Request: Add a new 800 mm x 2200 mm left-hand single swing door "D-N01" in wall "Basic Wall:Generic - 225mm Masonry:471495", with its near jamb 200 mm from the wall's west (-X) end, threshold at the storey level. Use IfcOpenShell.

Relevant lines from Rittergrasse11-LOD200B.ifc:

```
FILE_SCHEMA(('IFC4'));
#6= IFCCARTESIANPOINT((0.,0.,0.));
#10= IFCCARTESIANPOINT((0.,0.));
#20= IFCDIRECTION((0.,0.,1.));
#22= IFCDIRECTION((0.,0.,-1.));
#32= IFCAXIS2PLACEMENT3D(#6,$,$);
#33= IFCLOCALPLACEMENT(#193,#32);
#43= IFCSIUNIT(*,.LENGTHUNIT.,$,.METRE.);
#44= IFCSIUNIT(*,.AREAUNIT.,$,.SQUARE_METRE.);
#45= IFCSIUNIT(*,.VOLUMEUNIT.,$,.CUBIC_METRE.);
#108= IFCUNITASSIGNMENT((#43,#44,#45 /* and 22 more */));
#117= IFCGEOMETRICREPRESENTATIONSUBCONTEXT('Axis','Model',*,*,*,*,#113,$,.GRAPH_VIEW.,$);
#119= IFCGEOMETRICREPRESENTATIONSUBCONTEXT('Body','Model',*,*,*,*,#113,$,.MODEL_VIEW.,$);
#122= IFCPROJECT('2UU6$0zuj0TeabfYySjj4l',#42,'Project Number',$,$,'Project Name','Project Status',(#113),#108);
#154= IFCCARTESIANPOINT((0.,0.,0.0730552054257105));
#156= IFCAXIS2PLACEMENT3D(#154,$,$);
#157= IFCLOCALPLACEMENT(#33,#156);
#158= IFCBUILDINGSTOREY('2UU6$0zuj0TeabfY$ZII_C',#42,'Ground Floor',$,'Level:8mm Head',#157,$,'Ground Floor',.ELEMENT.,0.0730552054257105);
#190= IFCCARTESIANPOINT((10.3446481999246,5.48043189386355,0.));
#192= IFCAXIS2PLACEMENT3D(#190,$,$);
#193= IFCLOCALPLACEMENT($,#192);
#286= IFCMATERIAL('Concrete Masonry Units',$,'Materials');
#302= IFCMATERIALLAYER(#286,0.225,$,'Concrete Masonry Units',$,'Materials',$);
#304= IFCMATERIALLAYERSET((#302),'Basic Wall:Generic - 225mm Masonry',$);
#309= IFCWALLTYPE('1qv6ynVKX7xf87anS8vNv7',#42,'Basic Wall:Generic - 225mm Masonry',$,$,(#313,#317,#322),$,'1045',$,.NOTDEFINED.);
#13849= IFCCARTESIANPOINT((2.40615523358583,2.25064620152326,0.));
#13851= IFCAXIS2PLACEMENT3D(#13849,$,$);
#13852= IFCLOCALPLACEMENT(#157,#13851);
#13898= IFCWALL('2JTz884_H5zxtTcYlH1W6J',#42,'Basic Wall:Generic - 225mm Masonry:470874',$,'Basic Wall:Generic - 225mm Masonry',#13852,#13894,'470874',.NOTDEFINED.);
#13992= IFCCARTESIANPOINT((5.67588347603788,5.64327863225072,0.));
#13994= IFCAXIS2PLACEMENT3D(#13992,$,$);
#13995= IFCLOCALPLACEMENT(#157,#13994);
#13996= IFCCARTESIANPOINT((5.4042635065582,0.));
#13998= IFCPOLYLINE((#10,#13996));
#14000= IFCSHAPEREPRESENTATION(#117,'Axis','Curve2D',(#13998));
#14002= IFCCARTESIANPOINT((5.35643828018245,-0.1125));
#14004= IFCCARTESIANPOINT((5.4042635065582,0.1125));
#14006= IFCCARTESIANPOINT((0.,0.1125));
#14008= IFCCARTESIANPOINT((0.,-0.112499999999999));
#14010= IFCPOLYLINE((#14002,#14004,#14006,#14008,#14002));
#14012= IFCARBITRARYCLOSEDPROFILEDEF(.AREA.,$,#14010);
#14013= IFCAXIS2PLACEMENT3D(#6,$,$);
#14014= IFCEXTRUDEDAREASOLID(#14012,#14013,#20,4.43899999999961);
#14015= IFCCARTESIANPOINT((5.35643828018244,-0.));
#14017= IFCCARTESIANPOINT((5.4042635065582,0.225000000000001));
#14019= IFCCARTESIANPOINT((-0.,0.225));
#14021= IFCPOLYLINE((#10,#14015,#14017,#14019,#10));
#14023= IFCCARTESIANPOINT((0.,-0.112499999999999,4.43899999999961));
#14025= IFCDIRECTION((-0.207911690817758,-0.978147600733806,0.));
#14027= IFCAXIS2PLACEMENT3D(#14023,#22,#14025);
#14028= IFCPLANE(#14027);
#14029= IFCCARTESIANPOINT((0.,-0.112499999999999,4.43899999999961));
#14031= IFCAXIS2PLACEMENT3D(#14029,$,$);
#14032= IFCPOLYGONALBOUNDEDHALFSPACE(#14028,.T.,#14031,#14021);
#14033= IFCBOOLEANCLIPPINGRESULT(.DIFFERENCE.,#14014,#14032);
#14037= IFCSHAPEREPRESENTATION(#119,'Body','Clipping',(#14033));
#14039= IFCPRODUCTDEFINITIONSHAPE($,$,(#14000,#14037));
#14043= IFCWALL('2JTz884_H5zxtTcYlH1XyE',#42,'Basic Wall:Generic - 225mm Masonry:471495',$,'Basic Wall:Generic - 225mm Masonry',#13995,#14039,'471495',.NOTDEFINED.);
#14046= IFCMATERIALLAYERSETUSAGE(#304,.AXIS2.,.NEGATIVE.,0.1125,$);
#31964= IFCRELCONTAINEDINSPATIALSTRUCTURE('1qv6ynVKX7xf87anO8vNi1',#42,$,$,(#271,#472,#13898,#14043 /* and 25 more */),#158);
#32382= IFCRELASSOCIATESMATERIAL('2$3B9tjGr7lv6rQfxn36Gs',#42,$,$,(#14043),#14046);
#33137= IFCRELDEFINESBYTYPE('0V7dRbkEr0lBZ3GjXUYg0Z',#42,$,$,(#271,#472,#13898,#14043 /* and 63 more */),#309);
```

```python
import numpy as np
import ifcopenshell
import ifcopenshell.api.feature
import ifcopenshell.api.geometry
import ifcopenshell.api.root
import ifcopenshell.api.spatial
import ifcopenshell.geom
import ifcopenshell.util.element
import ifcopenshell.util.placement
import ifcopenshell.util.representation
import ifcopenshell.util.shape
import ifcopenshell.util.unit

model = ifcopenshell.open("Rittergrasse11-LOD200B.ifc")
unit_scale = ifcopenshell.util.unit.calculate_unit_scale(model)
settings = ifcopenshell.geom.settings()


def volume(element):
    """Net volume in cubic metres, openings subtracted."""
    shape = ifcopenshell.geom.create_shape(settings, element)
    return ifcopenshell.util.shape.get_volume(shape.geometry)


wall = model.by_guid("2JTz884_H5zxtTcYlH1XyE")
storey = ifcopenshell.util.element.get_container(wall, ifc_class="IfcBuildingStorey")
context = ifcopenshell.util.representation.get_context(model, "Model", "Body", "MODEL_VIEW")
before = volume(wall)

width, height, from_end, sill = 0.8, 2.2, 0.2, 0.0  # metres

# The wall runs along its own X axis, and the end named is its -X end.
wall_shape = ifcopenshell.geom.create_shape(settings, wall)
x, y, z = ifcopenshell.util.shape.get_vertices(wall_shape.geometry).T
start = x.min() + from_end
face, thickness = float(y.min()), float(y.max() - y.min())
wall_matrix = ifcopenshell.util.placement.get_local_placement(wall.ObjectPlacement)
level = ifcopenshell.util.placement.get_local_placement(storey.ObjectPlacement)[2, 3]


def in_wall(x, y):
    """Placement at x, y metres in the wall's axes, at sill height."""
    matrix = wall_matrix.copy()
    matrix[:, 3] = wall_matrix @ np.array([x / unit_scale, y / unit_scale, 0.0, 1.0])
    matrix[2, 3] = level + sill / unit_scale
    return matrix


# Opening: a box that overshoots both wall faces by 50 mm.
opening = ifcopenshell.api.root.create_entity(model, ifc_class="IfcOpeningElement", predefined_type="OPENING")
box = ifcopenshell.api.geometry.add_wall_representation(
    model, context=context, length=width, height=height, thickness=thickness + 0.1
)
ifcopenshell.api.geometry.assign_representation(model, product=opening, representation=box)
ifcopenshell.api.geometry.edit_object_placement(model, product=opening, matrix=in_wall(start, face - 0.05), is_si=False)
ifcopenshell.api.feature.add_feature(model, feature=opening, element=wall)

door = ifcopenshell.api.root.create_entity(model, ifc_class="IfcDoor", name="D-N01", predefined_type="DOOR")
door.OverallWidth, door.OverallHeight = width / unit_scale, height / unit_scale
door.OperationType = "SINGLE_SWING_LEFT"
body = ifcopenshell.api.geometry.add_door_representation(
    model,
    context=context,
    overall_width=door.OverallWidth,
    overall_height=door.OverallHeight,
    operation_type="SINGLE_SWING_LEFT",
    lining_properties={"LiningDepth": thickness / unit_scale, "ThresholdDepth": thickness / unit_scale},
)
ifcopenshell.api.geometry.assign_representation(model, product=door, representation=body)
ifcopenshell.api.spatial.assign_container(model, products=[door], relating_structure=storey)
ifcopenshell.api.feature.add_filling(model, opening=opening, element=door)

# The lining spans the wall, so the door starts at the wall face.
ifcopenshell.api.geometry.edit_object_placement(model, product=door, matrix=in_wall(start, face), is_si=False)

after = volume(wall)

print(f"wall volume {before:.3f} -> {after:.3f} m3")

model.write("Rittergrasse11-LOD200B_updated.ifc")
```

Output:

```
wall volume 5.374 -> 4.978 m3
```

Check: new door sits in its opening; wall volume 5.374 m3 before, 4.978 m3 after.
